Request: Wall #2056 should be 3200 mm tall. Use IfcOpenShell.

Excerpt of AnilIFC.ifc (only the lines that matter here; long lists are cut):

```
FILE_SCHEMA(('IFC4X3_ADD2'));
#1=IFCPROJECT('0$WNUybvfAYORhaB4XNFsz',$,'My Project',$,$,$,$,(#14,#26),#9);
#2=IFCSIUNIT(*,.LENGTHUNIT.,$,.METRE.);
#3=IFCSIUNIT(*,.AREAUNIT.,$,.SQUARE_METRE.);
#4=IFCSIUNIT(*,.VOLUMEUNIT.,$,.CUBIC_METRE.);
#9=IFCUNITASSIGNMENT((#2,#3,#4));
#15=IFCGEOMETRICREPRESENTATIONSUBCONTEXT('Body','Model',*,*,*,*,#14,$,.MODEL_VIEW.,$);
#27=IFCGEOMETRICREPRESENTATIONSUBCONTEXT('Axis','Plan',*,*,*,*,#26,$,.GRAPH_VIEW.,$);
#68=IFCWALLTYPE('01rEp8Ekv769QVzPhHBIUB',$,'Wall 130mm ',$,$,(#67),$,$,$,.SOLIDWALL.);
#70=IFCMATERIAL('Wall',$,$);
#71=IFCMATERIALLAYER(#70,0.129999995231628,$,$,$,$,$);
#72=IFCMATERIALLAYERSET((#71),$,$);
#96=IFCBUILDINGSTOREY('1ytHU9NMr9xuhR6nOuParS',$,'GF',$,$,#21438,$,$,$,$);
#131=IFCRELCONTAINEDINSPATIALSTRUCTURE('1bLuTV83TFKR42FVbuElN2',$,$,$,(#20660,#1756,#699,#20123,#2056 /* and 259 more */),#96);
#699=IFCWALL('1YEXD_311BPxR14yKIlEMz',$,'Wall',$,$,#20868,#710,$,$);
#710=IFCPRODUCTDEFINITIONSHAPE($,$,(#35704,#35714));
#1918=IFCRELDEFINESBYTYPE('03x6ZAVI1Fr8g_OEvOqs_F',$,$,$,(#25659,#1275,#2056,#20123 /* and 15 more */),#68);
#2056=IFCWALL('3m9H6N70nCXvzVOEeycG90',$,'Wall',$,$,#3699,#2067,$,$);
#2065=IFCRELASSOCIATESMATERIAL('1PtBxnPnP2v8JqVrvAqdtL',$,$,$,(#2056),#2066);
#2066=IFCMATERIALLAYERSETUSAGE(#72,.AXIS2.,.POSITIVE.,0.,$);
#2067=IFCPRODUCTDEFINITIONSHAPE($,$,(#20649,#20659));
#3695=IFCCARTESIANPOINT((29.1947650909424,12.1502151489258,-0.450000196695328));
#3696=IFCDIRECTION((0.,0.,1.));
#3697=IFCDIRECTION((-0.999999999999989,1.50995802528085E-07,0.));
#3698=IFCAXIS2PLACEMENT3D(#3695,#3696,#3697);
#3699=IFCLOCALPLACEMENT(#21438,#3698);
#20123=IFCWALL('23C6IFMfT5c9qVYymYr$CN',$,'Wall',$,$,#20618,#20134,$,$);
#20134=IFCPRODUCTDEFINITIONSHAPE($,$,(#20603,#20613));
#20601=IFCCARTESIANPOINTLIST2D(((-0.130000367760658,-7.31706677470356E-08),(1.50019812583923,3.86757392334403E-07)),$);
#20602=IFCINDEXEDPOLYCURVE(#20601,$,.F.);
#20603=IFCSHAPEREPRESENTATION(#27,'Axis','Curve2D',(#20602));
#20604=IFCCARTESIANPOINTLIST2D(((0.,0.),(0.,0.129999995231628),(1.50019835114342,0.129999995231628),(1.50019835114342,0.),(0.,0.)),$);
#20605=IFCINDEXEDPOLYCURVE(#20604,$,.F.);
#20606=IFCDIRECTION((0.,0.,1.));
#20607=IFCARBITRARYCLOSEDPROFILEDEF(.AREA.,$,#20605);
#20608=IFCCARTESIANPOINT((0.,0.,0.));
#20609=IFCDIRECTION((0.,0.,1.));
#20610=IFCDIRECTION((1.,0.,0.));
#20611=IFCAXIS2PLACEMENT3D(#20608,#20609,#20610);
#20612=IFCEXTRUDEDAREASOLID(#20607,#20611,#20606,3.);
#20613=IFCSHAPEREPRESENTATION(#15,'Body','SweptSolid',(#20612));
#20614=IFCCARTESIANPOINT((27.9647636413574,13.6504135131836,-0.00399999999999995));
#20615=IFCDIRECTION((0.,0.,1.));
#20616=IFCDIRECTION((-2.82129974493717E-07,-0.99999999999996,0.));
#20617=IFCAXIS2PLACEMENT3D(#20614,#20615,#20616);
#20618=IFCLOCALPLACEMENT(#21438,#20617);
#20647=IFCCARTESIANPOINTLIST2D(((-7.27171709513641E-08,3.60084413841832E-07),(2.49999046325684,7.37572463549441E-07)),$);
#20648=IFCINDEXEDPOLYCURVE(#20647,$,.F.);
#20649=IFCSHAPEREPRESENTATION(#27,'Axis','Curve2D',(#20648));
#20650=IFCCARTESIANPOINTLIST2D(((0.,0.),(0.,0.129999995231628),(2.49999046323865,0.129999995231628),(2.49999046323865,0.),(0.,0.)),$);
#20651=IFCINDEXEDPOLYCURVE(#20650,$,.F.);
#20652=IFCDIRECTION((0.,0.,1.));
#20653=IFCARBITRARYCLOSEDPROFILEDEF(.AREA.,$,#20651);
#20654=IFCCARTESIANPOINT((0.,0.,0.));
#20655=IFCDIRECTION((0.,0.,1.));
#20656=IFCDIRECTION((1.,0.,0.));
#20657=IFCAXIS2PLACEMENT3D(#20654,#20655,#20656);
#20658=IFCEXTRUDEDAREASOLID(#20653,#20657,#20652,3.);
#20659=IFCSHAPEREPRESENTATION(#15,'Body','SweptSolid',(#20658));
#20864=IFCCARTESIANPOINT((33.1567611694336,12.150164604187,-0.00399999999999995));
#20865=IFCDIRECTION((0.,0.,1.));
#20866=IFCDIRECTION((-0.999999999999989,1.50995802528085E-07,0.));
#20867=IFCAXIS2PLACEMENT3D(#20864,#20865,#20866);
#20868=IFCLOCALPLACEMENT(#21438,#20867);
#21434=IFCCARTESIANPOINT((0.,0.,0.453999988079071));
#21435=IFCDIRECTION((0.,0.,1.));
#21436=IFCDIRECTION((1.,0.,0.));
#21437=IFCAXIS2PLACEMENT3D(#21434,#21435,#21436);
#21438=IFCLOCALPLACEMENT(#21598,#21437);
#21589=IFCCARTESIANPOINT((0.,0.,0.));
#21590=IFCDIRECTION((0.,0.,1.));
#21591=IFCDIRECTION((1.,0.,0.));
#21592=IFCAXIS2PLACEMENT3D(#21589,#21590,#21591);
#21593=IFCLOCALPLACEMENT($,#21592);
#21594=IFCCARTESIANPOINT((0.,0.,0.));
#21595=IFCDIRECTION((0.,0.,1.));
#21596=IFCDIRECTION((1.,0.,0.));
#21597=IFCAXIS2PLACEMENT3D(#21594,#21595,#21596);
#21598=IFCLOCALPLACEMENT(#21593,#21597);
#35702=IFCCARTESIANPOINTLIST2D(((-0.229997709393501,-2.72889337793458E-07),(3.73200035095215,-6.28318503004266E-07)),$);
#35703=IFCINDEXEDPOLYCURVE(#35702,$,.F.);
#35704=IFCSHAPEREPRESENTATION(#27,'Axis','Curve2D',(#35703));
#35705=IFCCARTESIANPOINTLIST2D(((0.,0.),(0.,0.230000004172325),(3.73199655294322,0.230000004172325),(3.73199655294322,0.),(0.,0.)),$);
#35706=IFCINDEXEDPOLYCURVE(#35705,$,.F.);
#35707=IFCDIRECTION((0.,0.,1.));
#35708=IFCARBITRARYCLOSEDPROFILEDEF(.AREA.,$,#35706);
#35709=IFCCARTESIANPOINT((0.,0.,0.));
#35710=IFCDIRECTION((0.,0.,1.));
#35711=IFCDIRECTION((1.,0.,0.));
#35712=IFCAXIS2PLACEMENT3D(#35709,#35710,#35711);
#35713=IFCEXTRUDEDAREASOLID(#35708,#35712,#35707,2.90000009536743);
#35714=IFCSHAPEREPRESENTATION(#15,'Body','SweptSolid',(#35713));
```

```python
import ifcopenshell
import ifcopenshell.geom
import ifcopenshell.util.representation
import ifcopenshell.util.shape

model = ifcopenshell.open("AnilIFC.ifc")
settings = ifcopenshell.geom.settings()


def volume(element):
    """Net volume in cubic metres, openings subtracted."""
    shape = ifcopenshell.geom.create_shape(settings, element)
    return ifcopenshell.util.shape.get_volume(shape.geometry)


wall = model.by_id(2056)
before = volume(wall)

body = ifcopenshell.util.representation.get_representation(wall, "Model", "Body")
solid = body.Items[0]
old_height = solid.Depth
solid.Depth = 3.2
after = volume(wall)

print(f"height {old_height:g} -> {solid.Depth:g}, volume {before:.3f} -> {after:.3f} m3")

model.write("AnilIFC_updated.ifc")
```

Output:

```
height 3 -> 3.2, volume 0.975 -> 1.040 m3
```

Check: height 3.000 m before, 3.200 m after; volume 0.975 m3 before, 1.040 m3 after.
